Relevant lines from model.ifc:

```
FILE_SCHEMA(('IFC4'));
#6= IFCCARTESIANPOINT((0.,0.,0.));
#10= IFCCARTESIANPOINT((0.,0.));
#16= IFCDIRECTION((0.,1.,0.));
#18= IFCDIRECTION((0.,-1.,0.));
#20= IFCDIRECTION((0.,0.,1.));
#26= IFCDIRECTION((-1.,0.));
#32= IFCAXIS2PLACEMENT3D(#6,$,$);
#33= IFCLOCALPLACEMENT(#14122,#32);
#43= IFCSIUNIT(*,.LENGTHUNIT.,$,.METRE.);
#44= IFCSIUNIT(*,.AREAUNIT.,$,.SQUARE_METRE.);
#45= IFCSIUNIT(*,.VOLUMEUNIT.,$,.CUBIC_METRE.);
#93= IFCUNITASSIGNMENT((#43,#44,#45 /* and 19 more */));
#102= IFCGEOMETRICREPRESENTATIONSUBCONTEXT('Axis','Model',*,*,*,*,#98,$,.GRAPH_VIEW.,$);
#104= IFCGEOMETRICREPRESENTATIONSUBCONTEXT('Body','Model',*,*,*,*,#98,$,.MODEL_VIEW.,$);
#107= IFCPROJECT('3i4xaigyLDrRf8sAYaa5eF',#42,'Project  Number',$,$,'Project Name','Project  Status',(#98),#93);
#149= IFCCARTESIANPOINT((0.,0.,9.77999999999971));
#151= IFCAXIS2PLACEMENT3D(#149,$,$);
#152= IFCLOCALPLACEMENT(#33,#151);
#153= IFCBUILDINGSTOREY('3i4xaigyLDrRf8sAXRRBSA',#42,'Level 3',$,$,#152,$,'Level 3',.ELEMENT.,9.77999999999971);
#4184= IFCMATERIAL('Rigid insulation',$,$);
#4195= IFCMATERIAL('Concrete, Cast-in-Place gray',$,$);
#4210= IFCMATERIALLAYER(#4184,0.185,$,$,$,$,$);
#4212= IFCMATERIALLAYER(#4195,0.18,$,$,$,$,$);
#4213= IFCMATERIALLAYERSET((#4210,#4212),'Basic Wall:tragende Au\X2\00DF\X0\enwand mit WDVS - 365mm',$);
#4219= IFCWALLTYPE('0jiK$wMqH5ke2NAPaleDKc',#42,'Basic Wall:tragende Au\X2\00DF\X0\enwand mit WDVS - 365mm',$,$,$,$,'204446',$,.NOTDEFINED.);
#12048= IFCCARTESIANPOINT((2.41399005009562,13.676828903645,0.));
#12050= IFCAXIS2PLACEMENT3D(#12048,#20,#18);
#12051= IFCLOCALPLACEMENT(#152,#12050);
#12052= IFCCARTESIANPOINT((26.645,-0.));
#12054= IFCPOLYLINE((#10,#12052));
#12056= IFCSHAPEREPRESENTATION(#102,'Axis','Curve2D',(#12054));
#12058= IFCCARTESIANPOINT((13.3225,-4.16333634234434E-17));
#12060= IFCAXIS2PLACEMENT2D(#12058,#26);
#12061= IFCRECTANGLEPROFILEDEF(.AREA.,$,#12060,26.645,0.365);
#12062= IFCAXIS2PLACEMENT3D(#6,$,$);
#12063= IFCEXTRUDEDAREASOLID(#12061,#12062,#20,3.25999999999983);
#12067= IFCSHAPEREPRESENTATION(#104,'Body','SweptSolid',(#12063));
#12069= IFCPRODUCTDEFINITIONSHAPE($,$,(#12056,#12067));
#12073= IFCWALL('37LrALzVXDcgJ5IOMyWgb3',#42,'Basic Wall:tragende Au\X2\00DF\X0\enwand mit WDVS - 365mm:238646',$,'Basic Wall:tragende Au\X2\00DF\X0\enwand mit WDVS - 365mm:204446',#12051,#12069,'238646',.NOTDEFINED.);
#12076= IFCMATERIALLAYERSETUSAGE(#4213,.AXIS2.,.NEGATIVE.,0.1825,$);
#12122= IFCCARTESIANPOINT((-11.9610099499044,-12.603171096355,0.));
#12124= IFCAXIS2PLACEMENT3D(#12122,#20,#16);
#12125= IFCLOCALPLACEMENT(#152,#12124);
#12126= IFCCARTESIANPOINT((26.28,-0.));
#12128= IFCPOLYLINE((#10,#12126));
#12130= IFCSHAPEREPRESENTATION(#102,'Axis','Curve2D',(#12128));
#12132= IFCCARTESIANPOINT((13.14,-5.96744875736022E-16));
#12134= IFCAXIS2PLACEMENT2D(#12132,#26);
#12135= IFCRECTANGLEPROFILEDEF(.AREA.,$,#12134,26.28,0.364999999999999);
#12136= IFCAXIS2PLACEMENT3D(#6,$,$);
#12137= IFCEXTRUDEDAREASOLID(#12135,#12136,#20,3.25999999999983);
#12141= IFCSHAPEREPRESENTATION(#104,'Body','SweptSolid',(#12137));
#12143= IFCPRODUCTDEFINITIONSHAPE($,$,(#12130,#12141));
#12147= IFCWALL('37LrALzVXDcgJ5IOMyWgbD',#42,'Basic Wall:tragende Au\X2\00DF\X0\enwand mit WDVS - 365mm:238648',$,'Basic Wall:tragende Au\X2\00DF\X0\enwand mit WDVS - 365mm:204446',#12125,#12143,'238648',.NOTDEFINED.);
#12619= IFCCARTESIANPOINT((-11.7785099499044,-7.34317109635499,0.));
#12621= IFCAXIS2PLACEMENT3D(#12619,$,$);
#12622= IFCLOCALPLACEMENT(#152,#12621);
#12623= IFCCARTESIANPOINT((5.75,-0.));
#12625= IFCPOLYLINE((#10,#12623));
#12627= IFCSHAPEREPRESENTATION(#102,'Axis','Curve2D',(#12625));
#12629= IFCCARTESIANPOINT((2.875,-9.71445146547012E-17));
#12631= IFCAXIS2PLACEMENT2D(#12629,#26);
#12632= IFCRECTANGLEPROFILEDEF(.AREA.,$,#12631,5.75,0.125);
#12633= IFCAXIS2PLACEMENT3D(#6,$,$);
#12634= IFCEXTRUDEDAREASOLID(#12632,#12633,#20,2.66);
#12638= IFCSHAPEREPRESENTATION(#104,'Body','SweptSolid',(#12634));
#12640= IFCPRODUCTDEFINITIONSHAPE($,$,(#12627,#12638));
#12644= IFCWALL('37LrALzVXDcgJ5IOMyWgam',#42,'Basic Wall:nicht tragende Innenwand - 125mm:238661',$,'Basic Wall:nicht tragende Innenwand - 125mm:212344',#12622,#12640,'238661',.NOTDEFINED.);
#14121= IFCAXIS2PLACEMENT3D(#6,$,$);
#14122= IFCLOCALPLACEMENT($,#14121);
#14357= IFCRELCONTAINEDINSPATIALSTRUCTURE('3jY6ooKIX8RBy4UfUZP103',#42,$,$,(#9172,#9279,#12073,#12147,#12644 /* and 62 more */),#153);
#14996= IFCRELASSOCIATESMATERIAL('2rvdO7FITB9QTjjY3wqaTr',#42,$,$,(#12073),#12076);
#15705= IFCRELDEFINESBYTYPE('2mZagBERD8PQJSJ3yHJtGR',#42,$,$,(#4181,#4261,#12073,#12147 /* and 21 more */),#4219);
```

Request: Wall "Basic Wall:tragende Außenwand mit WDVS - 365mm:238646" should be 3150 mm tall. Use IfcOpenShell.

```python
import ifcopenshell
import ifcopenshell.geom
import ifcopenshell.util.representation
import ifcopenshell.util.shape

model = ifcopenshell.open("model.ifc")
settings = ifcopenshell.geom.settings()


def volume(element):
    """Net volume in cubic metres, openings subtracted."""
    shape = ifcopenshell.geom.create_shape(settings, element)
    return ifcopenshell.util.shape.get_volume(shape.geometry)


wall = model.by_id(12073)
before = volume(wall)

body = ifcopenshell.util.representation.get_representation(wall, "Model", "Body")
solid = body.Items[0]
old_height = solid.Depth
solid.Depth = 3.15
after = volume(wall)

print(f"height {old_height:g} -> {solid.Depth:g}, volume {before:.3f} -> {after:.3f} m3")

model.write("model_updated.ifc")
```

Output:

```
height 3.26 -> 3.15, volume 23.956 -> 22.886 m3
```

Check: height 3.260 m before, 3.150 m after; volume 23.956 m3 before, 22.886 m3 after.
